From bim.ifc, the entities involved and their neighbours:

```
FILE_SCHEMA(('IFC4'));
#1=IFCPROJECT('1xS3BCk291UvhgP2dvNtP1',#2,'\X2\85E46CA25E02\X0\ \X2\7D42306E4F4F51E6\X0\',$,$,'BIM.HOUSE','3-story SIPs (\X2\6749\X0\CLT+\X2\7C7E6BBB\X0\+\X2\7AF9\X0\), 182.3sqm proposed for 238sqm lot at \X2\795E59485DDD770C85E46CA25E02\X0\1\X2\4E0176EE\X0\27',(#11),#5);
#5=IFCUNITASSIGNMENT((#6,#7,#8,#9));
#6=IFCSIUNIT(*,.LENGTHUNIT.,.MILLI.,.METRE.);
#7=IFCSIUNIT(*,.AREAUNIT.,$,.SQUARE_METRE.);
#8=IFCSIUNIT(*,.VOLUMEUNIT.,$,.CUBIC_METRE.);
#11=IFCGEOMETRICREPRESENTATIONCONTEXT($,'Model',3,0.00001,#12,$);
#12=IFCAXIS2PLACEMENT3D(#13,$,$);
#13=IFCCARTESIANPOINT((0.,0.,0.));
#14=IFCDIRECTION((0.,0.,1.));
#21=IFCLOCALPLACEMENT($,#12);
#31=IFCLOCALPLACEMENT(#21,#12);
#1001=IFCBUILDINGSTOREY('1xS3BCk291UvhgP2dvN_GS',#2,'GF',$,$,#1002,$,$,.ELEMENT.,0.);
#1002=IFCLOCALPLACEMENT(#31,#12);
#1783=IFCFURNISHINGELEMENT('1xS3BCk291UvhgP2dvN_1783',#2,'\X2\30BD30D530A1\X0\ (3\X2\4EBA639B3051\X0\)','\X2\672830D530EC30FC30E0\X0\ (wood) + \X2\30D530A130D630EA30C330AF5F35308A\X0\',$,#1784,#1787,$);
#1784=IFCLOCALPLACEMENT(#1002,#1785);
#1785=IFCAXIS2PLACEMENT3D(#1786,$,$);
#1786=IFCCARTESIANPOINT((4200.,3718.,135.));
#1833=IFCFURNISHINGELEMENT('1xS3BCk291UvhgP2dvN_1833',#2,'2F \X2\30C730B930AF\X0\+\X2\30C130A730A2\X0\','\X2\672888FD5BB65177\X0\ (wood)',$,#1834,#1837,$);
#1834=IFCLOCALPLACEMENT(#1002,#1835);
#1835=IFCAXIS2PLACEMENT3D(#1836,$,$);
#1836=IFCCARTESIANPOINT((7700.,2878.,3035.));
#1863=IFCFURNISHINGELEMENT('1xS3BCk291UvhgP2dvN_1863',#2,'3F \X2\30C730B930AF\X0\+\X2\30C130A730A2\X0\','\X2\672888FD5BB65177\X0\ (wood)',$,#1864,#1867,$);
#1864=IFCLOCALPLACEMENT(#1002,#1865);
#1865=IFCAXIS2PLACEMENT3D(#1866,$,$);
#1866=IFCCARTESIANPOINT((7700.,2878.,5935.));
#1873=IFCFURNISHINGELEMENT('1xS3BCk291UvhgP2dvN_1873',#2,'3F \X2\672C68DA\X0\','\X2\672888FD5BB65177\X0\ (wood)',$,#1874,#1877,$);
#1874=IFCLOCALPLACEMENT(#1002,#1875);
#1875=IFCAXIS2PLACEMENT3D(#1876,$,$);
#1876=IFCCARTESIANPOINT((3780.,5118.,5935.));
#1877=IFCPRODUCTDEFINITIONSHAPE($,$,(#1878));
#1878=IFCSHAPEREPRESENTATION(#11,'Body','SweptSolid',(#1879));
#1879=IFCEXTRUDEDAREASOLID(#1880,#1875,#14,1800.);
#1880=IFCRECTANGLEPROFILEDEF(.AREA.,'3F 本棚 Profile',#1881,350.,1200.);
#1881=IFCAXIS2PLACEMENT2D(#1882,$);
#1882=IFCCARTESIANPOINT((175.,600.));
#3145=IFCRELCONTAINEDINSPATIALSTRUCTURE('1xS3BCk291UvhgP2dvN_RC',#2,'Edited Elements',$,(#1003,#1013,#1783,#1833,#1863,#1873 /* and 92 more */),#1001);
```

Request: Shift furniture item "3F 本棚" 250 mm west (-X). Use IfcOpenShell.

```python
import ifcopenshell
import ifcopenshell.api.geometry
import ifcopenshell.util.placement

model = ifcopenshell.open("bim.ifc")

item = model.by_guid("1xS3BCk291UvhgP2dvN_1873")
matrix = ifcopenshell.util.placement.get_local_placement(item.ObjectPlacement)
matrix[0, 3] -= 250.0
ifcopenshell.api.geometry.edit_object_placement(model, product=item, matrix=matrix, is_si=False)

print(ifcopenshell.util.placement.get_local_placement(item.ObjectPlacement).round(3) + 0.0)

model.write("bim_edited.ifc")
```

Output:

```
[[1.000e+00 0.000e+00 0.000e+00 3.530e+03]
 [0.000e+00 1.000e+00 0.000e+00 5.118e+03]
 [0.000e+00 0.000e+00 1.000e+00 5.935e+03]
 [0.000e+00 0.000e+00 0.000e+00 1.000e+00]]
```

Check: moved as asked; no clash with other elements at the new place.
